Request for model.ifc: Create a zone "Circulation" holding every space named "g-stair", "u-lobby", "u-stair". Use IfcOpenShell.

First a look at what the model holds.

```python
import ifcopenshell

model = ifcopenshell.open("model.ifc")
print(model.schema)
seen = {}
for space in model.by_type("IfcSpace"):
    seen[space.LongName] = seen.get(space.LongName, 0) + 1
for name, count in sorted(seen.items(), key=str):
    print(count, "x", name)
print("zones:", [z.Name for z in model.by_type("IfcZone")][:20])
```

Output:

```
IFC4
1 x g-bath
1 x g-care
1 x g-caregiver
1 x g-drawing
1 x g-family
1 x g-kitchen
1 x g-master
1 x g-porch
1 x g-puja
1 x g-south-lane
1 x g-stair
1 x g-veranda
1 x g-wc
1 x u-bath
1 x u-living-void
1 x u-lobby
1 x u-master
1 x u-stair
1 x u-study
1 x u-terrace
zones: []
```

```python
import ifcopenshell
import ifcopenshell.api.group
import ifcopenshell.api.root

model = ifcopenshell.open("model.ifc")

names = {"g-stair", "u-lobby", "u-stair"}
spaces = [s for s in model.by_type("IfcSpace") if s.LongName in names]

zone = ifcopenshell.api.root.create_entity(model, ifc_class="IfcZone", name="Circulation")
ifcopenshell.api.group.assign_group(model, products=spaces, group=zone)
print(len(spaces), "spaces in", zone.Name)

model.write("model_edited.ifc")
```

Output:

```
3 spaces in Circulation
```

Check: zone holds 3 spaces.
